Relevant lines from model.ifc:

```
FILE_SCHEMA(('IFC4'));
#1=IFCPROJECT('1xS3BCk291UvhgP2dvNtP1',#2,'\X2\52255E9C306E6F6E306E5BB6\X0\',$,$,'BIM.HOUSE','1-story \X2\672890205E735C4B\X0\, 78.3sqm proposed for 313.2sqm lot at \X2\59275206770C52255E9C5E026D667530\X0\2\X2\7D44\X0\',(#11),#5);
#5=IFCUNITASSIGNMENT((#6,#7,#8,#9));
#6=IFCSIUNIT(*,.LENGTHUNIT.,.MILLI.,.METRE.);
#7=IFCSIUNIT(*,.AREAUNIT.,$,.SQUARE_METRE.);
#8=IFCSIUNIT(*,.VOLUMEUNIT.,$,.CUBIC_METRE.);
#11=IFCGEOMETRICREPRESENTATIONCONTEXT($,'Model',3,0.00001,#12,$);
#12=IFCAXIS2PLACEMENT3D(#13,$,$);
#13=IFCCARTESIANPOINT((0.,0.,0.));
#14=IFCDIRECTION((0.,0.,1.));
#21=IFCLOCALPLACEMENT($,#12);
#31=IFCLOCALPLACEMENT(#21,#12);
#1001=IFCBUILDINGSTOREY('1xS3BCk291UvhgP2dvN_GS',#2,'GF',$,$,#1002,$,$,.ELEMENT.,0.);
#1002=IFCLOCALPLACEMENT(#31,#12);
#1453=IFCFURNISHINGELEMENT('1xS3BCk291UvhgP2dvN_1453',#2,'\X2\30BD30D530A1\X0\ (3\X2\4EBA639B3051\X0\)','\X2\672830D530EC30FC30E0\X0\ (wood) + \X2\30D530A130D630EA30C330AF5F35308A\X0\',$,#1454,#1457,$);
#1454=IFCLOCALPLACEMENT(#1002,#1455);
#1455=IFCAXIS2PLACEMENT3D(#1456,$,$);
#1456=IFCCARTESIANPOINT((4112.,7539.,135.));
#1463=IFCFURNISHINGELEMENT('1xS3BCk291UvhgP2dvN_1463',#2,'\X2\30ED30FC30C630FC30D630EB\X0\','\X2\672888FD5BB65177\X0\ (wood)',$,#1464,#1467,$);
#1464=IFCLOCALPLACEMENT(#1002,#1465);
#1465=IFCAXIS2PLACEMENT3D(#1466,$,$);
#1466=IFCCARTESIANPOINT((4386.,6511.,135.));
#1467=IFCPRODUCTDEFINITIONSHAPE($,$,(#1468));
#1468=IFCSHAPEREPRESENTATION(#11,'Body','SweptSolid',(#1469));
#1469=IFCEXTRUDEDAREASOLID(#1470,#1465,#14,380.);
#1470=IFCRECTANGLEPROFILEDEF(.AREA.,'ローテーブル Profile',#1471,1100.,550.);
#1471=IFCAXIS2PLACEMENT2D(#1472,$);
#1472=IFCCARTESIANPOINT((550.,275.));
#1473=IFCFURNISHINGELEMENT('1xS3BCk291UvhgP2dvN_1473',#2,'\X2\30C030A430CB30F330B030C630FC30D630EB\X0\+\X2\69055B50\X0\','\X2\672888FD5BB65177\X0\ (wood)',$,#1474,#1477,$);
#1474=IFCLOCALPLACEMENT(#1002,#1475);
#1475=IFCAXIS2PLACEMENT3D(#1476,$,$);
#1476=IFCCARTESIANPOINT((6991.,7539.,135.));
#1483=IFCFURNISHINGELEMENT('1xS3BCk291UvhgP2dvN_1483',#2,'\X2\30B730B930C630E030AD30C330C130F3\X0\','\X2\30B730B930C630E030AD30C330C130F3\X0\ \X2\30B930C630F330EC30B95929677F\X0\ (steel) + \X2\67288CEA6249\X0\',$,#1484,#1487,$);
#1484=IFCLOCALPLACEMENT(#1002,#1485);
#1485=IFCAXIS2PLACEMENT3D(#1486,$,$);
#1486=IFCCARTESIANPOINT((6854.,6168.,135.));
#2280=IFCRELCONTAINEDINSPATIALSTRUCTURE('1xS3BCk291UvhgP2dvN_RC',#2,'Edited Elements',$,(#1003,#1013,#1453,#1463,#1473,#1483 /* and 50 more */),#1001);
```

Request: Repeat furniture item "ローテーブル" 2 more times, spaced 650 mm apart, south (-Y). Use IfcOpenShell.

```python
import numpy as np
import ifcopenshell
import ifcopenshell.api.geometry
import ifcopenshell.api.root
import ifcopenshell.util.element
import ifcopenshell.util.placement
import ifcopenshell.util.unit

model = ifcopenshell.open("model.ifc")
unit_scale = ifcopenshell.util.unit.calculate_unit_scale(model)


def reuse_history(source, copy):
    """copy_class also copies each property set's owner history, people and application; keep the originals."""
    for rel in copy.IsDefinedBy:
        if rel.is_a("IfcRelDefinesByProperties") and (history := rel.RelatingPropertyDefinition.OwnerHistory):
            rel.RelatingPropertyDefinition.OwnerHistory = source.OwnerHistory
            ifcopenshell.util.element.remove_deep2(model, history)


source = model.by_guid("1xS3BCk291UvhgP2dvN_1463")
base = ifcopenshell.util.placement.get_local_placement(source.ObjectPlacement)
step = np.array([0.0, -1.0, 0.0]) * 0.65 / unit_scale

for i in range(1, 3):
    copy = ifcopenshell.api.root.copy_class(model, product=source)
    copy.Representation = ifcopenshell.util.element.copy_deep(
        model, source.Representation, exclude=["IfcGeometricRepresentationContext", "IfcRepresentationMap"]
    )
    reuse_history(source, copy)
    matrix = base.copy()
    matrix[:3, 3] += i * step
    print("added at", matrix[:3, 3].round(3) + 0.0)
    ifcopenshell.api.geometry.edit_object_placement(model, product=copy, matrix=matrix, is_si=False)

model.write("model_v2.ifc")
```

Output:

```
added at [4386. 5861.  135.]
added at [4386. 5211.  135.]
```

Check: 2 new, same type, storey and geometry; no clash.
